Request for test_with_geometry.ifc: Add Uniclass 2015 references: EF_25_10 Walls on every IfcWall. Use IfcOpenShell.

First a look at what the model holds.

```python
import ifcopenshell

model = ifcopenshell.open("test_with_geometry.ifc")
print(model.schema)
print("classifications:", [c.Name for c in model.by_type("IfcClassification")])
for ifc_class in ("IfcDoor", "IfcRoof", "IfcStair", "IfcWall", "IfcWindow"):
    print(ifc_class, len(model.by_type(ifc_class)))
```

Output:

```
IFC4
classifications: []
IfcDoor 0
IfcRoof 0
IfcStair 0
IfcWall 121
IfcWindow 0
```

```python
import ifcopenshell
import ifcopenshell.api.classification

model = ifcopenshell.open("test_with_geometry.ifc")

system = ifcopenshell.api.classification.add_classification(model, classification="Uniclass 2015")

codes = {
    "IfcWall": ("EF_25_10", "Walls"),
}
for ifc_class, (code, name) in codes.items():
    products = model.by_type(ifc_class)
    ifcopenshell.api.classification.add_reference(
        model, products=products, classification=system, identification=code, name=name
    )
    print(code, len(products))

model.write("test_with_geometry_edited.ifc")
```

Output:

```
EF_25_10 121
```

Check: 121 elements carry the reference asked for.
